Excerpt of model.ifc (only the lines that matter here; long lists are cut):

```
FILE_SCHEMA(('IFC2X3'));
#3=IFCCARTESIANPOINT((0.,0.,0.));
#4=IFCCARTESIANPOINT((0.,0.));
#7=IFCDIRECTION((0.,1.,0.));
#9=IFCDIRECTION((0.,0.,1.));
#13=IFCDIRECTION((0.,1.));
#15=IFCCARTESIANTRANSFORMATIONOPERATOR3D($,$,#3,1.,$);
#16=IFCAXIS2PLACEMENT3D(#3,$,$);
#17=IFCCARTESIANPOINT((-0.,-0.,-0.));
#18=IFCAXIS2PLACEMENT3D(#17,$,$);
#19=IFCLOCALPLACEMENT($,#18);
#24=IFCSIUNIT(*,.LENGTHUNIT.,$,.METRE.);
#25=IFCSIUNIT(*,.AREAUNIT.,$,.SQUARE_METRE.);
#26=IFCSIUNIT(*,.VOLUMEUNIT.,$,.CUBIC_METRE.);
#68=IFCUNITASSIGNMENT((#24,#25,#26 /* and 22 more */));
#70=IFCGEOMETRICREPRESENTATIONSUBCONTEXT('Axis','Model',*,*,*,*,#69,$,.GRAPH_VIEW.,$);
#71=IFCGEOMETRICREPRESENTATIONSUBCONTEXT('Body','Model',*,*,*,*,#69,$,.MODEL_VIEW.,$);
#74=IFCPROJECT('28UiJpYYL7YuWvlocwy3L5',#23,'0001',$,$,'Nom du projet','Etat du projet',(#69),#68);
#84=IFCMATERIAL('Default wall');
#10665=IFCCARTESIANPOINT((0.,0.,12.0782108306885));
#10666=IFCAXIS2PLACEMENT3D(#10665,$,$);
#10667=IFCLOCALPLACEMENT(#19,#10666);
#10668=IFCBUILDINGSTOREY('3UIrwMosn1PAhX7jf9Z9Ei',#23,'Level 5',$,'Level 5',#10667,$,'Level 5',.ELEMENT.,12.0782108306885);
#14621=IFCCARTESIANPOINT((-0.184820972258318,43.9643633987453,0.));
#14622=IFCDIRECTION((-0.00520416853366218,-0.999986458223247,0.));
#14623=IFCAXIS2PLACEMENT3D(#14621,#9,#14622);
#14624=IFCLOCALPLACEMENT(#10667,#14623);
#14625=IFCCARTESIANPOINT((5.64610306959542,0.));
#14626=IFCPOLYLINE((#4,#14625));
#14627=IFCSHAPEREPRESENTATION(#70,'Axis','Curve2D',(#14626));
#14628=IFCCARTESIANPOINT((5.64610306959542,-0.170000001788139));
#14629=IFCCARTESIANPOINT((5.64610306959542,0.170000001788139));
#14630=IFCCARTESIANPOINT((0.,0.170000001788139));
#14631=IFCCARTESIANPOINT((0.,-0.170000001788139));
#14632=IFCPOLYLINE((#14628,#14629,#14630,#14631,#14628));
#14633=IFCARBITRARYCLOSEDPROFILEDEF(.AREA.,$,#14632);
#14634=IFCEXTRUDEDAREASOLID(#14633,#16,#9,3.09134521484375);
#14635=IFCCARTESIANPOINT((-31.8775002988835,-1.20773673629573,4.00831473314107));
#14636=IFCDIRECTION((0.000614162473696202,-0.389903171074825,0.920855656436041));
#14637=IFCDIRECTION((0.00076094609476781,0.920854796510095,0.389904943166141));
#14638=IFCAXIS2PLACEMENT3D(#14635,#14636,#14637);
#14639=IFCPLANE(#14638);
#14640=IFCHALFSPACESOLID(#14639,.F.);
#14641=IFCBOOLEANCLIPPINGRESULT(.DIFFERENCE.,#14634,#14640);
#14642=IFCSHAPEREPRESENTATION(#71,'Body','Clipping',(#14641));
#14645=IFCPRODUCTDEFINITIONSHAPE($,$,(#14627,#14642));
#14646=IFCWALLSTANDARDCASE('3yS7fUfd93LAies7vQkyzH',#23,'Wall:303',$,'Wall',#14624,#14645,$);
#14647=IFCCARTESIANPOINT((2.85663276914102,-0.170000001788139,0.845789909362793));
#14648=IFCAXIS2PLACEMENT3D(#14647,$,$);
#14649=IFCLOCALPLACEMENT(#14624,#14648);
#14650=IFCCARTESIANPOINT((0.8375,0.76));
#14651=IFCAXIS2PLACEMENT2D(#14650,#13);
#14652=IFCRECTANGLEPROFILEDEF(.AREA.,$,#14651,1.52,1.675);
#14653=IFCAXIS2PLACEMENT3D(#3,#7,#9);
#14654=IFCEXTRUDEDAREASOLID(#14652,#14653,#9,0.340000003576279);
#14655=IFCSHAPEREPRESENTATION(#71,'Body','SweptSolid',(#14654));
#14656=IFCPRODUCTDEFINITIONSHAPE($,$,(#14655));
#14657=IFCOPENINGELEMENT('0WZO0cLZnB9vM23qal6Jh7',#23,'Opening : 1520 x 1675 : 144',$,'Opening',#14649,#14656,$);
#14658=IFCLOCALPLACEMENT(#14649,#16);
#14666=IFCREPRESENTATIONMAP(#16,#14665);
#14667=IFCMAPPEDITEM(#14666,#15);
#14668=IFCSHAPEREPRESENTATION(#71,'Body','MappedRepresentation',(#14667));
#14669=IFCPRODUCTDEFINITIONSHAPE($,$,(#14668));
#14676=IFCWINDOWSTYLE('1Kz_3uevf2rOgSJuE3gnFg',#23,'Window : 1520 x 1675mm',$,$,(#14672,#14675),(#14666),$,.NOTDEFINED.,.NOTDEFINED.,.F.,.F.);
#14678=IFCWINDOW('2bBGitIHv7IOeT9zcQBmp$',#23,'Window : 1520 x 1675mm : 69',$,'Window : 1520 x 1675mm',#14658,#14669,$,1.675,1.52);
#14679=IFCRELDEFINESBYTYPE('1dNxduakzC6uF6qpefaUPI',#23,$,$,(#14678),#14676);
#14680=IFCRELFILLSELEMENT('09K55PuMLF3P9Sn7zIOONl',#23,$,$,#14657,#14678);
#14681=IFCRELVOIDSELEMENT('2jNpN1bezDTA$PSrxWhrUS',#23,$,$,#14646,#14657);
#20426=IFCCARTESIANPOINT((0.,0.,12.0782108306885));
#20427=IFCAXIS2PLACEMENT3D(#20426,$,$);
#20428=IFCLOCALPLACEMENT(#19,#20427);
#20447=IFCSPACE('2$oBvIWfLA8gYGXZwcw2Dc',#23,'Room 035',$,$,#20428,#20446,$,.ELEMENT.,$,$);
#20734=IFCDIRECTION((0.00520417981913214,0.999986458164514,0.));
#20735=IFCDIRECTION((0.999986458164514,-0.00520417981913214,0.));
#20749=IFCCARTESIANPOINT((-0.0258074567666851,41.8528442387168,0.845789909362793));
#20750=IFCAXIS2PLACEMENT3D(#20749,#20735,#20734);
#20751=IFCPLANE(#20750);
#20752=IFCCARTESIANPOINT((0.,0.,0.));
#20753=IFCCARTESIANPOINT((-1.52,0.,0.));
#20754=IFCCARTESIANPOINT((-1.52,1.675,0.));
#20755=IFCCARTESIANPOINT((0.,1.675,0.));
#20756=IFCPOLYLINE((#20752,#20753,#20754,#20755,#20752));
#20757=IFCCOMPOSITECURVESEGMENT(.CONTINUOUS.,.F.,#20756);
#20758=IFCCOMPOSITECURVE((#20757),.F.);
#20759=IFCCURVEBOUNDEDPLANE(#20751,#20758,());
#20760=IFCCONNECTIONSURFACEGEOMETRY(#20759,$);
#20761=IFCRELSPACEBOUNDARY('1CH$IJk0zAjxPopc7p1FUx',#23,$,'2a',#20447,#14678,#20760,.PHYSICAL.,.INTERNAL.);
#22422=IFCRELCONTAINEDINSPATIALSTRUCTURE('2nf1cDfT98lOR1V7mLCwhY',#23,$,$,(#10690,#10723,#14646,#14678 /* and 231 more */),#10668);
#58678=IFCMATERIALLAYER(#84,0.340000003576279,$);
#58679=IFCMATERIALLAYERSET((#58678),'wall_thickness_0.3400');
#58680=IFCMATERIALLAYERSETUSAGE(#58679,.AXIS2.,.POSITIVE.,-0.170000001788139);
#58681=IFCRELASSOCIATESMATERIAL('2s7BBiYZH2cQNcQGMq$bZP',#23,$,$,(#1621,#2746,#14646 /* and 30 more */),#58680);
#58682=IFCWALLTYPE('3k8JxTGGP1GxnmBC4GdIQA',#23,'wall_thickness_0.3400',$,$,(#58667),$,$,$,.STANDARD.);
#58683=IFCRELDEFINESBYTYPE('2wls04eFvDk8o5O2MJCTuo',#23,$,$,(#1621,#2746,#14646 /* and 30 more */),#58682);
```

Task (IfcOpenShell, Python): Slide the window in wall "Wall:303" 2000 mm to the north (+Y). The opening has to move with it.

```python
import numpy as np
import ifcopenshell
import ifcopenshell.api.geometry
import ifcopenshell.util.placement
import ifcopenshell.util.unit

model = ifcopenshell.open("model.ifc")
unit_scale = ifcopenshell.util.unit.calculate_unit_scale(model)

window = model.by_guid("2bBGitIHv7IOeT9zcQBmp$")
opening = window.FillsVoids[0].RelatingOpeningElement
wall = opening.VoidsElements[0].RelatingBuildingElement

wall_matrix = ifcopenshell.util.placement.get_local_placement(wall.ObjectPlacement)
shift = wall_matrix[:3, 0] * -2 / unit_scale
before = ifcopenshell.util.placement.get_local_placement(window.ObjectPlacement)[:3, 3].copy()

# The window is placed relative to its opening, so it follows when the opening moves.
matrix = ifcopenshell.util.placement.get_local_placement(opening.ObjectPlacement)
matrix[:3, 3] += shift
ifcopenshell.api.geometry.edit_object_placement(
    model, product=opening, matrix=matrix, is_si=False, should_transform_children=True
)

# Space boundary surfaces are stored in each space's coordinates; move them too.
for rel in window.ProvidesBoundaries:
    if not rel.ConnectionGeometry:
        continue
    surface = rel.ConnectionGeometry.SurfaceOnRelatingElement.BasisSurface
    space_matrix = ifcopenshell.util.placement.get_local_placement(rel.RelatingSpace.ObjectPlacement)
    point = np.array(surface.Position.Location.Coordinates) + space_matrix[:3, :3].T @ shift
    surface.Position = model.createIfcAxis2Placement3D(
        model.createIfcCartesianPoint(point.tolist()), surface.Position.Axis, surface.Position.RefDirection
    )

after = ifcopenshell.util.placement.get_local_placement(window.ObjectPlacement)[:3, 3]
print("window moved by", (after - before).round(3) + 0.0)

model.write("model-out.ifc")
```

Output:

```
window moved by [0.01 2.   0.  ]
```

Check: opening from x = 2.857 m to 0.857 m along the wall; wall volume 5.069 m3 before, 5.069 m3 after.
